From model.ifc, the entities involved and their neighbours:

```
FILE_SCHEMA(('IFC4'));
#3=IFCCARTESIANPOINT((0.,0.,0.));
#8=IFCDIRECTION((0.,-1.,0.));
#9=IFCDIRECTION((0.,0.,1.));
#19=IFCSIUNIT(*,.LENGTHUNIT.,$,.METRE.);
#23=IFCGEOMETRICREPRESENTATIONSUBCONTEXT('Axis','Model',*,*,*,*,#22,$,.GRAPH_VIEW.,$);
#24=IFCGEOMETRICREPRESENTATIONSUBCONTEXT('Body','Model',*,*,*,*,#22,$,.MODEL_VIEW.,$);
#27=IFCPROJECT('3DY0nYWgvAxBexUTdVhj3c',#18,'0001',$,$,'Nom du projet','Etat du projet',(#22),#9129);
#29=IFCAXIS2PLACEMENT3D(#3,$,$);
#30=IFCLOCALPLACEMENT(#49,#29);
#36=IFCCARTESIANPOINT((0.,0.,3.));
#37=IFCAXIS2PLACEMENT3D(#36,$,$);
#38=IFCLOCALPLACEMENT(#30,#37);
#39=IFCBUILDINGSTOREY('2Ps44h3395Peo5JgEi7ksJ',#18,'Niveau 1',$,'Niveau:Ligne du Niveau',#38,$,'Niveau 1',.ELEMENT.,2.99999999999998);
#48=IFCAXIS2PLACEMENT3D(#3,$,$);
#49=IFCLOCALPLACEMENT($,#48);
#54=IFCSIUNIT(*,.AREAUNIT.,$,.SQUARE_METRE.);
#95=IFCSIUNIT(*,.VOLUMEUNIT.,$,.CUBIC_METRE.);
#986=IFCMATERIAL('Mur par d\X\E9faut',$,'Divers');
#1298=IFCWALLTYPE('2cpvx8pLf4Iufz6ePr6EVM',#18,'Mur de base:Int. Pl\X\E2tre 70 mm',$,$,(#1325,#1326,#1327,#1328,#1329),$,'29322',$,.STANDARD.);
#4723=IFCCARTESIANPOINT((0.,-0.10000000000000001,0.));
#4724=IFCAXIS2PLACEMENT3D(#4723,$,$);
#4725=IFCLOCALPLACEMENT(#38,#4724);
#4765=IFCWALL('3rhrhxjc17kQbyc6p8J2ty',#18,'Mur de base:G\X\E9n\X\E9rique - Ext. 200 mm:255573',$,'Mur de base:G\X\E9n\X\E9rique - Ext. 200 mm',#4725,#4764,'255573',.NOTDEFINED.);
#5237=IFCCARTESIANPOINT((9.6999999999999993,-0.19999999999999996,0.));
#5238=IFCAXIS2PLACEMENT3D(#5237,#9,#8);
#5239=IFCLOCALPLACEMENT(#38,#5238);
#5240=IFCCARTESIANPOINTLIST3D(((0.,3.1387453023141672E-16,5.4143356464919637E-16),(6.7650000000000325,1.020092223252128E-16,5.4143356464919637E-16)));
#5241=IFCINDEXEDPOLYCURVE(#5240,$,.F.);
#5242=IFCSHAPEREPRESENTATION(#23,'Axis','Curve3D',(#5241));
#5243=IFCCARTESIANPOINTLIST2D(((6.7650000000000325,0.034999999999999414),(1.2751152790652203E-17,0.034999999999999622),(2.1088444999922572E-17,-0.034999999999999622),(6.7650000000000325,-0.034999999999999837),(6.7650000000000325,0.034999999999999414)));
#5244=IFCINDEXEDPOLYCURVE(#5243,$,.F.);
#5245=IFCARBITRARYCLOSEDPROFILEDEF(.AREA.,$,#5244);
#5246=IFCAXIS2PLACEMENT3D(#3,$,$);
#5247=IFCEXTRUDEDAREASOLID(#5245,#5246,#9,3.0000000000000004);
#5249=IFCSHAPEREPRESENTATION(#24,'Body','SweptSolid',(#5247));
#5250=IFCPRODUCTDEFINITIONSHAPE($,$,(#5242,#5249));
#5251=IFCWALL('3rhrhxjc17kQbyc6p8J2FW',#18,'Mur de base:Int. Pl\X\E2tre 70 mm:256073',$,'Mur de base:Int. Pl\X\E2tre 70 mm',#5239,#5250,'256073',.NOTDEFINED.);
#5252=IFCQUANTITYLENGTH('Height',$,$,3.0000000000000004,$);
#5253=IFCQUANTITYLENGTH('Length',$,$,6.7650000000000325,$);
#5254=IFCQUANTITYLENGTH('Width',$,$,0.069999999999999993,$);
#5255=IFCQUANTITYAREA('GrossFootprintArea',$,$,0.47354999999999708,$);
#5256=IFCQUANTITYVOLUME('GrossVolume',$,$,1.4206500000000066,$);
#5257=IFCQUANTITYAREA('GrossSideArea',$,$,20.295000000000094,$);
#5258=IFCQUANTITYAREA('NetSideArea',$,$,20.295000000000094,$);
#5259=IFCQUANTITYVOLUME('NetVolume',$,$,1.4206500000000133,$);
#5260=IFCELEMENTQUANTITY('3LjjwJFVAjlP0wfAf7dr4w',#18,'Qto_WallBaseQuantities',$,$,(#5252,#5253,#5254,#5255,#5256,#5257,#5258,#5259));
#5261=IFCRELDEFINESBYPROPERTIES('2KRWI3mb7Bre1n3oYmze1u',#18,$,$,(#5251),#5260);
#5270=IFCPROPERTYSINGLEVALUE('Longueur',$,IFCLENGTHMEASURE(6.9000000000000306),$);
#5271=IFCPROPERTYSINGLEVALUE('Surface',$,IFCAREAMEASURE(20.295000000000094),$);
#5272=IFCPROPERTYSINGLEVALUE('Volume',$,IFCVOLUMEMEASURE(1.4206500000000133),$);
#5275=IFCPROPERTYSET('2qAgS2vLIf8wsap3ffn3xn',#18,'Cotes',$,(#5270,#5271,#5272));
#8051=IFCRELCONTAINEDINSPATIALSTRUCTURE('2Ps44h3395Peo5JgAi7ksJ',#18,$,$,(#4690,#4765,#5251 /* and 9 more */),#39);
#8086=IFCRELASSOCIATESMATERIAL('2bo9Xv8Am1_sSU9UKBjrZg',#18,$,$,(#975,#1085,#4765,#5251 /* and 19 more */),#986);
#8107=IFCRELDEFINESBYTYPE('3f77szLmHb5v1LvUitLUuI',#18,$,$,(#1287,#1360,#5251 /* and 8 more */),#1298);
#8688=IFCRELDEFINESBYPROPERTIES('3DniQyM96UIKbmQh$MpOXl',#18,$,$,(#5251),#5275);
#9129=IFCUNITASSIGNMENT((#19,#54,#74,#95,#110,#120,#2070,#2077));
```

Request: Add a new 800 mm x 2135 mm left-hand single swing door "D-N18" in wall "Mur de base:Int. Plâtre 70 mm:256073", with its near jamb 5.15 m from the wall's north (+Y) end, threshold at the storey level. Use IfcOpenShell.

```python
import numpy as np
import ifcopenshell
import ifcopenshell.api.feature
import ifcopenshell.api.geometry
import ifcopenshell.api.pset
import ifcopenshell.api.root
import ifcopenshell.api.spatial
import ifcopenshell.geom
import ifcopenshell.util.element
import ifcopenshell.util.placement
import ifcopenshell.util.representation
import ifcopenshell.util.shape
import ifcopenshell.util.unit

model = ifcopenshell.open("model.ifc")
unit_scale = ifcopenshell.util.unit.calculate_unit_scale(model)
area_scale = ifcopenshell.util.unit.calculate_unit_scale(model, "AREAUNIT")
volume_scale = ifcopenshell.util.unit.calculate_unit_scale(model, "VOLUMEUNIT")
settings = ifcopenshell.geom.settings()


def volume(element):
    """Net volume in cubic metres, openings subtracted."""
    shape = ifcopenshell.geom.create_shape(settings, element)
    return ifcopenshell.util.shape.get_volume(shape.geometry)


wall = model.by_guid("3rhrhxjc17kQbyc6p8J2FW")
storey = ifcopenshell.util.element.get_container(wall, ifc_class="IfcBuildingStorey")
context = ifcopenshell.util.representation.get_context(model, "Model", "Body", "MODEL_VIEW")
before = volume(wall)

width, height, from_end, sill = 0.8, 2.135, 5.15, 0.0  # metres

# The wall runs along its own X axis, and the end named is its -X end.
wall_shape = ifcopenshell.geom.create_shape(settings, wall)
x, y, z = ifcopenshell.util.shape.get_vertices(wall_shape.geometry).T
start = x.min() + from_end
face, thickness = float(y.min()), float(y.max() - y.min())
wall_matrix = ifcopenshell.util.placement.get_local_placement(wall.ObjectPlacement)
level = ifcopenshell.util.placement.get_local_placement(storey.ObjectPlacement)[2, 3]


def in_wall(x, y):
    """Placement at x, y metres in the wall's axes, at sill height."""
    matrix = wall_matrix.copy()
    matrix[:, 3] = wall_matrix @ np.array([x / unit_scale, y / unit_scale, 0.0, 1.0])
    matrix[2, 3] = level + sill / unit_scale
    return matrix


# Opening: a box that overshoots both wall faces by 50 mm.
opening = ifcopenshell.api.root.create_entity(model, ifc_class="IfcOpeningElement", predefined_type="OPENING")
box = ifcopenshell.api.geometry.add_wall_representation(
    model, context=context, length=width, height=height, thickness=thickness + 0.1
)
ifcopenshell.api.geometry.assign_representation(model, product=opening, representation=box)
ifcopenshell.api.geometry.edit_object_placement(model, product=opening, matrix=in_wall(start, face - 0.05), is_si=False)
ifcopenshell.api.feature.add_feature(model, feature=opening, element=wall)

door = ifcopenshell.api.root.create_entity(model, ifc_class="IfcDoor", name="D-N18", predefined_type="DOOR")
door.OverallWidth, door.OverallHeight = width / unit_scale, height / unit_scale
door.OperationType = "SINGLE_SWING_LEFT"
body = ifcopenshell.api.geometry.add_door_representation(
    model,
    context=context,
    overall_width=door.OverallWidth,
    overall_height=door.OverallHeight,
    operation_type="SINGLE_SWING_LEFT",
    lining_properties={"LiningDepth": thickness / unit_scale, "ThresholdDepth": thickness / unit_scale},
)
ifcopenshell.api.geometry.assign_representation(model, product=door, representation=body)
ifcopenshell.api.spatial.assign_container(model, products=[door], relating_structure=storey)
ifcopenshell.api.feature.add_filling(model, opening=opening, element=door)

# The lining spans the wall, so the door starts at the wall face.
ifcopenshell.api.geometry.edit_object_placement(model, product=door, matrix=in_wall(start, face), is_si=False)

after = volume(wall)

# Update the wall's stored quantities.
qto = model.by_id(ifcopenshell.util.element.get_pset(wall, "Qto_WallBaseQuantities", should_inherit=False)["id"])
ifcopenshell.api.pset.edit_qto(model, qto=qto, properties={
    "NetSideArea": after / thickness / area_scale,
    "NetVolume": after / volume_scale,
})
pset = model.by_id(ifcopenshell.util.element.get_pset(wall, "Cotes", should_inherit=False)["id"])
ifcopenshell.api.pset.edit_pset(model, pset=pset, properties={
    "Surface": model.create_entity("IfcAreaMeasure", after / thickness / area_scale),
    "Volume": model.create_entity("IfcVolumeMeasure", after / volume_scale),
})

print(f"wall volume {before:.3f} -> {after:.3f} m3")

model.write("model_rev.ifc")
```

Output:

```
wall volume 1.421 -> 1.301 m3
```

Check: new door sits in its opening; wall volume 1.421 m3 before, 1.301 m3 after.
